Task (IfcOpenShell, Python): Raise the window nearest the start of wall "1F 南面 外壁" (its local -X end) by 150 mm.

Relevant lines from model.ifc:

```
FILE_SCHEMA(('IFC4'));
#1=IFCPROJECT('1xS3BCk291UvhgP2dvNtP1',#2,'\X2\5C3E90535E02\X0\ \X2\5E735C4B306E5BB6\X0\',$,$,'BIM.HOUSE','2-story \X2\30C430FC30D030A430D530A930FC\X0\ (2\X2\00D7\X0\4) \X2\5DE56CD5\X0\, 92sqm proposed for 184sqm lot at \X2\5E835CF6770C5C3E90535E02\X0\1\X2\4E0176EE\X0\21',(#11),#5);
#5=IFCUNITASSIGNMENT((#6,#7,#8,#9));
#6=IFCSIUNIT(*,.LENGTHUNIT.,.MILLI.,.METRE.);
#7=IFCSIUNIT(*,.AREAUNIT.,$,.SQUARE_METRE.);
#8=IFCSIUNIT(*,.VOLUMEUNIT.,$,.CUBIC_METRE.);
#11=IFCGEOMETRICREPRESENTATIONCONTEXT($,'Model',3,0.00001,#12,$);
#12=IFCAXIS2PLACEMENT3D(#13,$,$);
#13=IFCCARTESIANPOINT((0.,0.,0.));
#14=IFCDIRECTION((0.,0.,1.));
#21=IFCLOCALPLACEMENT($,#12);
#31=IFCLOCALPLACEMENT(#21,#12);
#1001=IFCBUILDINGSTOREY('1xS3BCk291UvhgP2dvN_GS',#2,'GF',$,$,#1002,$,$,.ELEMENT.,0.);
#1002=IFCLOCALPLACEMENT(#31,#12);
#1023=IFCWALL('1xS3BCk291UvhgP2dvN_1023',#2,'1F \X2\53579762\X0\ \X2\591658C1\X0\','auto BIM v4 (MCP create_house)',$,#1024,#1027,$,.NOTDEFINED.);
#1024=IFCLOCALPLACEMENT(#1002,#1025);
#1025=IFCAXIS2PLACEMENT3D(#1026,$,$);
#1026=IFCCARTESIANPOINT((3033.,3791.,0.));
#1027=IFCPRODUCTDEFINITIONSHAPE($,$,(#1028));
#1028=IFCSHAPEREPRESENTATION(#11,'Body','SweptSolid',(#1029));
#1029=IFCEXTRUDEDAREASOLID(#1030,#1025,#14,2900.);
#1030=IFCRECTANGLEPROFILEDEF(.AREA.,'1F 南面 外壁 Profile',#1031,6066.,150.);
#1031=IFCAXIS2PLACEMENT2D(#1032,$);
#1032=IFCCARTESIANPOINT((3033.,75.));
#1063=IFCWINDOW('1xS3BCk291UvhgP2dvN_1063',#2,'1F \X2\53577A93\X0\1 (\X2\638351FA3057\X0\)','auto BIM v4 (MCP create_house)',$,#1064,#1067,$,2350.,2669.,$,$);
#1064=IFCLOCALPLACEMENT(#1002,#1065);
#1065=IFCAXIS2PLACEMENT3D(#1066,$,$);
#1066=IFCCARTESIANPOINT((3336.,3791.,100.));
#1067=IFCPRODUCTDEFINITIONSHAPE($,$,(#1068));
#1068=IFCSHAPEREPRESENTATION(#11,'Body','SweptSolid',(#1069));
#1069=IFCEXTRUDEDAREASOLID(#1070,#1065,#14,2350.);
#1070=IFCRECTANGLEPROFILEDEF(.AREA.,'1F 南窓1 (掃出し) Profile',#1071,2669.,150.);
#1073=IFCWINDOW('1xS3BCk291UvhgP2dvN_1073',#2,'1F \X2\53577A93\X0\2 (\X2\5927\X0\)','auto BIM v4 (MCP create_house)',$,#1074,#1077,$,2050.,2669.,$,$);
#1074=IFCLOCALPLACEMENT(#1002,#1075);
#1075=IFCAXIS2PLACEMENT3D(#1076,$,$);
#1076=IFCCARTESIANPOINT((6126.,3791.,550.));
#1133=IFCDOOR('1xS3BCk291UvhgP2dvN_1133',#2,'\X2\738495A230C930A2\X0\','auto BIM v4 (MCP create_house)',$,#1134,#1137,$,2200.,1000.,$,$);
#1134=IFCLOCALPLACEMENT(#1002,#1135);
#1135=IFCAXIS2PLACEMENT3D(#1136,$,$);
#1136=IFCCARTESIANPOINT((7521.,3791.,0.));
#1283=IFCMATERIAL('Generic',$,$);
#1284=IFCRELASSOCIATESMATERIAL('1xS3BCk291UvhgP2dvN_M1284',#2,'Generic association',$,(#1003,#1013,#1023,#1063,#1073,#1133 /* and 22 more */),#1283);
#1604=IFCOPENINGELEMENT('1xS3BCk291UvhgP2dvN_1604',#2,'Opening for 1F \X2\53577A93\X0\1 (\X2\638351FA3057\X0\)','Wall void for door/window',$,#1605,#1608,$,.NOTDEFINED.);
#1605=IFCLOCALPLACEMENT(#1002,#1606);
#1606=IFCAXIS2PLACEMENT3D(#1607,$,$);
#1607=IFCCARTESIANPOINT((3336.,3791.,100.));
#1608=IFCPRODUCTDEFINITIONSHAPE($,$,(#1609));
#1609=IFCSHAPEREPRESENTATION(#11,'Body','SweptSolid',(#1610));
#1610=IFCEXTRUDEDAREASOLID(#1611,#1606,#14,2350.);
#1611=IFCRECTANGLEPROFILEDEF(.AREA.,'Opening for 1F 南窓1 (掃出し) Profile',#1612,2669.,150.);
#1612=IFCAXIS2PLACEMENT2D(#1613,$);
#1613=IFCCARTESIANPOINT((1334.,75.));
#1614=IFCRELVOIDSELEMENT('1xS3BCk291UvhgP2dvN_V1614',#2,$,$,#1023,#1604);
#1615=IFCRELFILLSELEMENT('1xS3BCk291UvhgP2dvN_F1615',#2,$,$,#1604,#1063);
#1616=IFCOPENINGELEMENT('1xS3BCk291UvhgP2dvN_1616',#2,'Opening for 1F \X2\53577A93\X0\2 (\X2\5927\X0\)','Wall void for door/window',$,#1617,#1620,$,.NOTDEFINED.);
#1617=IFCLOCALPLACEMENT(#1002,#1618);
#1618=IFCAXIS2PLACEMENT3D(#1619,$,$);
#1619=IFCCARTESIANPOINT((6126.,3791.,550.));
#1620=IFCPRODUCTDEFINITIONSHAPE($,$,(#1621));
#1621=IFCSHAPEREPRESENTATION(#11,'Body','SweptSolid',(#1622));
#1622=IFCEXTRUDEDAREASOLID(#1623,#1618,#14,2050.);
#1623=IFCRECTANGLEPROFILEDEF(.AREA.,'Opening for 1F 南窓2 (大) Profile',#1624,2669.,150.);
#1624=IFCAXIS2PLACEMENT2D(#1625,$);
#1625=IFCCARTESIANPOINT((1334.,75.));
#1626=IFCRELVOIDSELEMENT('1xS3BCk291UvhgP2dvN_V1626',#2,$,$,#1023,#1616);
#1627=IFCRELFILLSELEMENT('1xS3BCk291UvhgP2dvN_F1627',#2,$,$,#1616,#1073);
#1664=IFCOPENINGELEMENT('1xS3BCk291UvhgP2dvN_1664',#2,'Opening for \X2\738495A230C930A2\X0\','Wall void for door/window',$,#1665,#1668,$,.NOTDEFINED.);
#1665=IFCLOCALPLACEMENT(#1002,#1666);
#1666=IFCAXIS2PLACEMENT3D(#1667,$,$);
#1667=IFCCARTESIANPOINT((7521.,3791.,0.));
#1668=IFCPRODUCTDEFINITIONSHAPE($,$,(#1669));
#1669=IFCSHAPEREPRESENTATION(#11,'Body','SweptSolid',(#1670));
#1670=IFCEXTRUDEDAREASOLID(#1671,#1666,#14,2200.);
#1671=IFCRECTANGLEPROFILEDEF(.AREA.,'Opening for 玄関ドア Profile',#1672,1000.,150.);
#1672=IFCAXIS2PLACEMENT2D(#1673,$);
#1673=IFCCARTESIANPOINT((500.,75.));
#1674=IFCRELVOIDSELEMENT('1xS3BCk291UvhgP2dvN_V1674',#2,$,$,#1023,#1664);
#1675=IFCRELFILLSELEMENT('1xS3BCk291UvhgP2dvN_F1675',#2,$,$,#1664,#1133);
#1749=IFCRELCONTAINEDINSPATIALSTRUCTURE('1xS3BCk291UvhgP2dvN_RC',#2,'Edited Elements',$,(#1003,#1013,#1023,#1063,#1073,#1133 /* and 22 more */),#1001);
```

```python
import numpy as np
import ifcopenshell
import ifcopenshell.api.geometry
import ifcopenshell.util.placement
import ifcopenshell.util.unit

model = ifcopenshell.open("model.ifc")
unit_scale = ifcopenshell.util.unit.calculate_unit_scale(model)

window = model.by_guid("1xS3BCk291UvhgP2dvN_1063")
opening = window.FillsVoids[0].RelatingOpeningElement
dz = 150.0

shift = np.array([0.0, 0.0, dz])
# The window is not placed relative to its opening, so move both.
for product in (opening, window):
    matrix = ifcopenshell.util.placement.get_local_placement(product.ObjectPlacement)
    matrix[:3, 3] += shift
    ifcopenshell.api.geometry.edit_object_placement(model, product=product, matrix=matrix, is_si=False)

print(f"moved by {dz * unit_scale:+.3f} m")

model.write("model-out.ifc")
```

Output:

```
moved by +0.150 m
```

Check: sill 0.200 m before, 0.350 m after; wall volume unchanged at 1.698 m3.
